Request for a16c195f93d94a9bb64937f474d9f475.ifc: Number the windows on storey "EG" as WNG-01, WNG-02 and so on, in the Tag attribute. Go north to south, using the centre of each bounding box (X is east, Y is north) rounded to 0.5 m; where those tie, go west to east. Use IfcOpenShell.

First a look at what the model holds.

```python
import ifcopenshell
import ifcopenshell.util.element
import ifcopenshell.util.placement

model = ifcopenshell.open("a16c195f93d94a9bb64937f474d9f475.ifc")
print(model.schema)
storey = next(s for s in model.by_type("IfcBuildingStorey") if s.Name == "EG")
windows = [e for e in ifcopenshell.util.element.get_decomposition(storey) if e.is_a("IfcWindow")]
for e in sorted(windows, key=lambda e: e.id()):
    origin = ifcopenshell.util.placement.get_local_placement(e.ObjectPlacement)[:3, 3]
    print(e.id(), e.Tag, e.Name, origin.round(2) + 0.0, sep=" | ")
```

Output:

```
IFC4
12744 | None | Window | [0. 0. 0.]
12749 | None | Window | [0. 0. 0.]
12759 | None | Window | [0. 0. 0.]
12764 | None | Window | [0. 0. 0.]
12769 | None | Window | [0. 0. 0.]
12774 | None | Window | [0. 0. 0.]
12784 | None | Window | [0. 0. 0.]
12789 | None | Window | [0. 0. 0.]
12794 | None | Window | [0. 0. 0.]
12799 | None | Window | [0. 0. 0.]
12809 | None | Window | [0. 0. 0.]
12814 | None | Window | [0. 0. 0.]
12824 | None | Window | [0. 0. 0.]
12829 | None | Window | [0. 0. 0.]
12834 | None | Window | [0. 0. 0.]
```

```python
import ifcopenshell
import ifcopenshell.geom
import ifcopenshell.util.element
import ifcopenshell.util.shape

model = ifcopenshell.open("a16c195f93d94a9bb64937f474d9f475.ifc")
settings = ifcopenshell.geom.settings()
settings.set("use-world-coords", True)


def centre(element):
    shape = ifcopenshell.geom.create_shape(settings, element)
    return ifcopenshell.util.shape.get_bbox_centroid(shape.geometry)


storey = next(s for s in model.by_type("IfcBuildingStorey") if s.Name == "EG")
windows = [e for e in ifcopenshell.util.element.get_decomposition(storey) if e.is_a("IfcWindow")]

# Insertion points can sit at a corner or the storey origin, so sort by the geometry (in metres).
centres = {e: centre(e) for e in windows}
windows.sort(key=lambda e: (-round(centres[e][1] / 0.5), centres[e][0]))

for i, e in enumerate(windows, start=1):
    number = f"WNG-{i:02d}"
    e.Tag = number
    print(e.id(), number)

model.write("a16c195f93d94a9bb64937f474d9f475_edited.ifc")
```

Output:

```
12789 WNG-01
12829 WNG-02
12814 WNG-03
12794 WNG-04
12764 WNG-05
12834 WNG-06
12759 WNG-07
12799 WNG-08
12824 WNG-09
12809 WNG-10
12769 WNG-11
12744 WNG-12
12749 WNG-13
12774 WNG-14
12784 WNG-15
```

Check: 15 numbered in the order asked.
